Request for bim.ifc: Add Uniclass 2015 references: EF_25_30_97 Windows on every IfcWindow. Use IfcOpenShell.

First a look at what the model holds.

```python
import ifcopenshell

model = ifcopenshell.open("bim.ifc")
print(model.schema)
print("classifications:", [c.Name for c in model.by_type("IfcClassification")])
for ifc_class in ("IfcDoor", "IfcRoof", "IfcStair", "IfcWall", "IfcWindow"):
    print(ifc_class, len(model.by_type(ifc_class)))
```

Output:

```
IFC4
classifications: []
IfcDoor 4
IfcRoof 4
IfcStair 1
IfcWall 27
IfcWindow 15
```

```python
import ifcopenshell
import ifcopenshell.api.classification

model = ifcopenshell.open("bim.ifc")

system = ifcopenshell.api.classification.add_classification(model, classification="Uniclass 2015")

codes = {
    "IfcWindow": ("EF_25_30_97", "Windows"),
}
for ifc_class, (code, name) in codes.items():
    products = model.by_type(ifc_class)
    ifcopenshell.api.classification.add_reference(
        model, products=products, classification=system, identification=code, name=name
    )
    print(code, len(products))

model.write("bim_edited.ifc")
```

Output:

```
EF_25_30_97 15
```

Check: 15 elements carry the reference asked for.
